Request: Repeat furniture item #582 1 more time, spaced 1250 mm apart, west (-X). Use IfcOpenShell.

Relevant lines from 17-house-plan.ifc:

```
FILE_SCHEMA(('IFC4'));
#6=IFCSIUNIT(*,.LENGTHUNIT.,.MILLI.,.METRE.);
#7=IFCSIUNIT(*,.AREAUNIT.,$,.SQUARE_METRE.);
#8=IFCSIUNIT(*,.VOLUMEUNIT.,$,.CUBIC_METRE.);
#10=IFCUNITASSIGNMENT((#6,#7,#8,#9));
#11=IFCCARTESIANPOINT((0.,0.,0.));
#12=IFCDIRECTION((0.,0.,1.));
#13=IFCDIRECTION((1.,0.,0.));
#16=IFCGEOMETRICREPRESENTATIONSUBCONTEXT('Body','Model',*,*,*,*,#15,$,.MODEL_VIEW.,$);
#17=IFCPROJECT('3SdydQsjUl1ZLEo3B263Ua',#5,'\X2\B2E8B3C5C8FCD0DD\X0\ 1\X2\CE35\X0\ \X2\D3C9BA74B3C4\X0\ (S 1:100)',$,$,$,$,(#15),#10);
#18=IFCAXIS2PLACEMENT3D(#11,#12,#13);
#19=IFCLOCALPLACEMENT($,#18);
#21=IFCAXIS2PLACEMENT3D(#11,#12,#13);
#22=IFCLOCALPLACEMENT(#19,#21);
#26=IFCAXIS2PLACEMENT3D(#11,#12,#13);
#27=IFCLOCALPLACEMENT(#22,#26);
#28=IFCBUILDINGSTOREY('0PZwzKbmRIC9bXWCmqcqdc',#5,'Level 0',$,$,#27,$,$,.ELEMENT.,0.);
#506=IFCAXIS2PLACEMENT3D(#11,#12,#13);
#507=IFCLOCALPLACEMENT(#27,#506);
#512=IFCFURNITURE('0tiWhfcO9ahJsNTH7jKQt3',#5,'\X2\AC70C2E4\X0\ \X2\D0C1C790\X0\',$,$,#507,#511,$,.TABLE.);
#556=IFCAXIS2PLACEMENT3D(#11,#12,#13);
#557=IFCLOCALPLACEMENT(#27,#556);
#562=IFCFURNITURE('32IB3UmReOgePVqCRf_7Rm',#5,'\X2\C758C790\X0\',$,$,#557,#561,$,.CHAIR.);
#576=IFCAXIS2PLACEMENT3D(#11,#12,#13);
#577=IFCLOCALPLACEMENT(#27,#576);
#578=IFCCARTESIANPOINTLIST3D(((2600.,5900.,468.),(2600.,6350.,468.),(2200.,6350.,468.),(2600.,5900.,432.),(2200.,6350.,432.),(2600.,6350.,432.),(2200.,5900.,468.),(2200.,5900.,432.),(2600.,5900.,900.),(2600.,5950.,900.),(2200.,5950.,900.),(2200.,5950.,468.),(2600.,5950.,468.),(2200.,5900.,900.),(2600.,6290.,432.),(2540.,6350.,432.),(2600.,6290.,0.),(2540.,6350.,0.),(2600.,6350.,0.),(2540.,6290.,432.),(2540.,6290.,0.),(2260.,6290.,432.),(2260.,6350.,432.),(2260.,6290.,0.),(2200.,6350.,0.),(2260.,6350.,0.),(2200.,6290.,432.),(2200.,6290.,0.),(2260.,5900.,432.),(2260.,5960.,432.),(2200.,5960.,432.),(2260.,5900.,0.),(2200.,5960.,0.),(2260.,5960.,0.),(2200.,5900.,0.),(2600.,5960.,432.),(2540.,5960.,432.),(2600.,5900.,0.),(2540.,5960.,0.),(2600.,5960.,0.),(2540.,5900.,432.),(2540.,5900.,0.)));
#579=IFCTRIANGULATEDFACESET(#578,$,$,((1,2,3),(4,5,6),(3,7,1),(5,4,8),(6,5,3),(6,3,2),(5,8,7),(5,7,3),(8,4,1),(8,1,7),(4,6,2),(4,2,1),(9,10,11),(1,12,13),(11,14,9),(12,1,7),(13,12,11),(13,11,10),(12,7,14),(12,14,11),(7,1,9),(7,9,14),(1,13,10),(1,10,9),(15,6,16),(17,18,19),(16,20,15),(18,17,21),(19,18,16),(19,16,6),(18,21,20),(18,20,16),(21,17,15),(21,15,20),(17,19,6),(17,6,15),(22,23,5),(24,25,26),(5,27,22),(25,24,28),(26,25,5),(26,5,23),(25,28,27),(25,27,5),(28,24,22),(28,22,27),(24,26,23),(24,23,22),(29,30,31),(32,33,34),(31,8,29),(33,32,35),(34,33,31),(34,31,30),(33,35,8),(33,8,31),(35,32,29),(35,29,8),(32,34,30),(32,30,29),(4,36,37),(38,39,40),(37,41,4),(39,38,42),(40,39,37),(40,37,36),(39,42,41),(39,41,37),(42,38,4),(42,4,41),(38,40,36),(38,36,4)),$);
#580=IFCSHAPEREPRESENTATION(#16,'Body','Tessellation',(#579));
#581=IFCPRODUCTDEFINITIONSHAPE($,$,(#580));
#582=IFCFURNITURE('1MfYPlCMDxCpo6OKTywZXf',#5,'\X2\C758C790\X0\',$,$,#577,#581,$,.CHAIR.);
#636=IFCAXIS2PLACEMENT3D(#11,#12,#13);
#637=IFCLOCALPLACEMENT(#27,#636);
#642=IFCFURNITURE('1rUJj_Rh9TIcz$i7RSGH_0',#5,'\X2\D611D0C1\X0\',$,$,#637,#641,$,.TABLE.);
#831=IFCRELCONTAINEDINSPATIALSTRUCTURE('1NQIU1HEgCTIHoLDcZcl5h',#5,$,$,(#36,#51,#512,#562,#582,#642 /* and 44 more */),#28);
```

```python
import numpy as np
import ifcopenshell
import ifcopenshell.api.geometry
import ifcopenshell.api.root
import ifcopenshell.util.element
import ifcopenshell.util.placement

model = ifcopenshell.open("17-house-plan.ifc")


def reuse_history(source, copy):
    """copy_class also copies each property set's owner history, people and application; keep the originals."""
    for rel in copy.IsDefinedBy:
        if rel.is_a("IfcRelDefinesByProperties") and (history := rel.RelatingPropertyDefinition.OwnerHistory):
            rel.RelatingPropertyDefinition.OwnerHistory = source.OwnerHistory
            ifcopenshell.util.element.remove_deep2(model, history)


source = model.by_id(582)
base = ifcopenshell.util.placement.get_local_placement(source.ObjectPlacement)
step = np.array([-1.0, 0.0, 0.0]) * 1250.0

for i in range(1, 2):
    copy = ifcopenshell.api.root.copy_class(model, product=source)
    copy.Representation = ifcopenshell.util.element.copy_deep(
        model, source.Representation, exclude=["IfcGeometricRepresentationContext", "IfcRepresentationMap"]
    )
    reuse_history(source, copy)
    matrix = base.copy()
    matrix[:3, 3] += i * step
    print("added at", matrix[:3, 3].round(3) + 0.0)
    ifcopenshell.api.geometry.edit_object_placement(model, product=copy, matrix=matrix, is_si=False)

model.write("17-house-plan-out.ifc")
```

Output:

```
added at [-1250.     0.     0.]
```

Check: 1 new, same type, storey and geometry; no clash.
